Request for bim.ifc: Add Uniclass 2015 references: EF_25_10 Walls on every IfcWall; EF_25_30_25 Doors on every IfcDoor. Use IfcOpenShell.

First a look at what the model holds.

```python
import ifcopenshell

model = ifcopenshell.open("bim.ifc")
print(model.schema)
print("classifications:", [c.Name for c in model.by_type("IfcClassification")])
for ifc_class in ("IfcDoor", "IfcRoof", "IfcStair", "IfcWall", "IfcWindow"):
    print(ifc_class, len(model.by_type(ifc_class)))
```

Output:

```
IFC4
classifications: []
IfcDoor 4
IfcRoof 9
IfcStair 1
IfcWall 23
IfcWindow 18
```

```python
import ifcopenshell
import ifcopenshell.api.classification

model = ifcopenshell.open("bim.ifc")

system = ifcopenshell.api.classification.add_classification(model, classification="Uniclass 2015")

codes = {
    "IfcWall": ("EF_25_10", "Walls"),
    "IfcDoor": ("EF_25_30_25", "Doors"),
}
for ifc_class, (code, name) in codes.items():
    products = model.by_type(ifc_class)
    ifcopenshell.api.classification.add_reference(
        model, products=products, classification=system, identification=code, name=name
    )
    print(code, len(products))

model.write("bim_edited.ifc")
```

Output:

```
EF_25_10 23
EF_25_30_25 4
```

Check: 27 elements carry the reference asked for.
